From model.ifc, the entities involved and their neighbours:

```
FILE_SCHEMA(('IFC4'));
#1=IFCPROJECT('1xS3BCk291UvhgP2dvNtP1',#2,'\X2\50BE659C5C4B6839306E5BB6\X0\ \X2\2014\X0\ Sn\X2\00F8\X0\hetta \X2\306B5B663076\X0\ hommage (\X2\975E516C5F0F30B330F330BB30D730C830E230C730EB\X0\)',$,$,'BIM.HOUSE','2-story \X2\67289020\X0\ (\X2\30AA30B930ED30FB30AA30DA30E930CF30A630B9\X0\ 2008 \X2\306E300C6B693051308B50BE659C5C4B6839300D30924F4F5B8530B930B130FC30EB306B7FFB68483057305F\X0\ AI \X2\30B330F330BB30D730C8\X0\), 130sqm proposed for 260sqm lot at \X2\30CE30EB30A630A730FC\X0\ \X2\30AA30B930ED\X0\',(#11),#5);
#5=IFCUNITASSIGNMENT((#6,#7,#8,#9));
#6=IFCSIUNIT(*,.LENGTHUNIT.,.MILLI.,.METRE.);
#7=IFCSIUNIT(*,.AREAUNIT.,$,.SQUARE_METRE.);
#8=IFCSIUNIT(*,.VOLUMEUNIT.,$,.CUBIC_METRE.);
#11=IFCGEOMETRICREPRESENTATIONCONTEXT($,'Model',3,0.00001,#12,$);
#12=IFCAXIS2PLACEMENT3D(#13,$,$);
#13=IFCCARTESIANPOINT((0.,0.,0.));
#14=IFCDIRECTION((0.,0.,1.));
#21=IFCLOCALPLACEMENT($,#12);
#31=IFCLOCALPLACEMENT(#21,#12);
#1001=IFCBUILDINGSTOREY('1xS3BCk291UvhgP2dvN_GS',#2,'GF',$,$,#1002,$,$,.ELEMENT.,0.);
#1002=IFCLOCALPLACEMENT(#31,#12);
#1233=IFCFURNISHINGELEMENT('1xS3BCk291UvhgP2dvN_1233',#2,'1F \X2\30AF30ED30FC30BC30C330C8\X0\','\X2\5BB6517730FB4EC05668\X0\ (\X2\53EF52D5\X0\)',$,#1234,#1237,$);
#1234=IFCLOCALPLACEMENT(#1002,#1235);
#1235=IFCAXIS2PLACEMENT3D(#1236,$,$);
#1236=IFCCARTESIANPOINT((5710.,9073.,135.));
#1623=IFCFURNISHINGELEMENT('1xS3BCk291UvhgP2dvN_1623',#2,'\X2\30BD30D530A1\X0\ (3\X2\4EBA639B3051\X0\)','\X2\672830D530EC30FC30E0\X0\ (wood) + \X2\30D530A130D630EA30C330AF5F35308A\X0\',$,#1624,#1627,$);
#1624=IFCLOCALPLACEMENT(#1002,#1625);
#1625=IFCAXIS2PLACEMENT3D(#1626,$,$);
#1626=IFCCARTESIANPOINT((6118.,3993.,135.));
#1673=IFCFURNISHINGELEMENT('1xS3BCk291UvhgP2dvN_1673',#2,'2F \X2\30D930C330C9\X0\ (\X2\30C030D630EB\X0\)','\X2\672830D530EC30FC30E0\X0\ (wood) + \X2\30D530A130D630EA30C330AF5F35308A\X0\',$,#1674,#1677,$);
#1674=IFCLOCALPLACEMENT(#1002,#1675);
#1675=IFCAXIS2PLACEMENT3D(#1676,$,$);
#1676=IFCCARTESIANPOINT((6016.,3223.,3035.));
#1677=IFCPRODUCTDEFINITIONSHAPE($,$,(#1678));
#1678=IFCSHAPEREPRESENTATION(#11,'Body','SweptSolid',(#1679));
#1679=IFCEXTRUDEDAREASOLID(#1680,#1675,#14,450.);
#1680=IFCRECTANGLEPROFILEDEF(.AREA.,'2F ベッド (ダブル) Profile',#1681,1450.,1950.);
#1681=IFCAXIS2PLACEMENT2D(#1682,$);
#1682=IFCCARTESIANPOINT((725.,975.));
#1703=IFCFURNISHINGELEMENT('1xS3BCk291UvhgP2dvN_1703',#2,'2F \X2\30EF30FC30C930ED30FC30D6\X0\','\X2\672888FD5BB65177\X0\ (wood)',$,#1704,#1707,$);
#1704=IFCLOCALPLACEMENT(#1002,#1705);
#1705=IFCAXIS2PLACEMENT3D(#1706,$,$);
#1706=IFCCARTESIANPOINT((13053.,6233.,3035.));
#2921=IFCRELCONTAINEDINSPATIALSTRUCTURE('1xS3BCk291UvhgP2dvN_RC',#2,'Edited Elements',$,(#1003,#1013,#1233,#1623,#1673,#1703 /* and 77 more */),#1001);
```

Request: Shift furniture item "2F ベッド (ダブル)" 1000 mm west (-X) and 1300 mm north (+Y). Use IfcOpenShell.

```python
import ifcopenshell
import ifcopenshell.api.geometry
import ifcopenshell.util.placement

model = ifcopenshell.open("model.ifc")

item = model.by_guid("1xS3BCk291UvhgP2dvN_1673")
matrix = ifcopenshell.util.placement.get_local_placement(item.ObjectPlacement)
matrix[0, 3] -= 1000.0
matrix[1, 3] += 1300.0
ifcopenshell.api.geometry.edit_object_placement(model, product=item, matrix=matrix, is_si=False)

print(ifcopenshell.util.placement.get_local_placement(item.ObjectPlacement).round(3) + 0.0)

model.write("model_rev.ifc")
```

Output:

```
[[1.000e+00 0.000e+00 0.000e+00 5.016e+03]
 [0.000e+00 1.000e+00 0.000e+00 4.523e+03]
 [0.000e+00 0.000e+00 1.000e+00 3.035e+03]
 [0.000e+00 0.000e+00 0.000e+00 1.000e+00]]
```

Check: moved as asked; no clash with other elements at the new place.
